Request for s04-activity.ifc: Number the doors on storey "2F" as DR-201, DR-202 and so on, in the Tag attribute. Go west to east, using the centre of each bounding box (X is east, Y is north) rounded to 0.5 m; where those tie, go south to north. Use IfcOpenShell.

First a look at what the model holds.

```python
import ifcopenshell
import ifcopenshell.util.element
import ifcopenshell.util.placement

model = ifcopenshell.open("s04-activity.ifc")
print(model.schema)
storey = next(s for s in model.by_type("IfcBuildingStorey") if s.Name == "2F")
doors = [e for e in ifcopenshell.util.element.get_decomposition(storey) if e.is_a("IfcDoor")]
for e in sorted(doors, key=lambda e: e.id()):
    origin = ifcopenshell.util.placement.get_local_placement(e.ObjectPlacement)[:3, 3]
    print(e.id(), e.Tag, e.Name, origin.round(2) + 0.0, sep=" | ")
```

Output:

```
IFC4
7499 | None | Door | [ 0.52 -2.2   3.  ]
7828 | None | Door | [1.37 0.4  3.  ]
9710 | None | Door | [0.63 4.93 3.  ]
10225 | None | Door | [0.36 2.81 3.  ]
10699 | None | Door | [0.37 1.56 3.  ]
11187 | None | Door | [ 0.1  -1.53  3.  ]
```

```python
import ifcopenshell
import ifcopenshell.geom
import ifcopenshell.util.element
import ifcopenshell.util.shape

model = ifcopenshell.open("s04-activity.ifc")
settings = ifcopenshell.geom.settings()
settings.set("use-world-coords", True)


def centre(element):
    shape = ifcopenshell.geom.create_shape(settings, element)
    return ifcopenshell.util.shape.get_bbox_centroid(shape.geometry)


storey = next(s for s in model.by_type("IfcBuildingStorey") if s.Name == "2F")
doors = [e for e in ifcopenshell.util.element.get_decomposition(storey) if e.is_a("IfcDoor")]

# Insertion points can sit at a corner or the storey origin, so sort by the geometry (in metres).
centres = {e: centre(e) for e in doors}
doors.sort(key=lambda e: (round(centres[e][0] / 0.5), centres[e][1]))

for i, e in enumerate(doors, start=1):
    number = f"DR-2{i:02d}"
    e.Tag = number
    print(e.id(), number)

model.write("s04-activity-out.ifc")
```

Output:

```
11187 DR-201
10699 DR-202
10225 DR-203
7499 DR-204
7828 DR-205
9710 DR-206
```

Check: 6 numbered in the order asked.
